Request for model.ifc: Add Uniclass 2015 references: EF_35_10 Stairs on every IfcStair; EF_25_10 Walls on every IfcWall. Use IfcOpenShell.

First a look at what the model holds.

```python
import ifcopenshell

model = ifcopenshell.open("model.ifc")
print(model.schema)
print("classifications:", [c.Name for c in model.by_type("IfcClassification")])
for ifc_class in ("IfcDoor", "IfcRoof", "IfcStair", "IfcWall", "IfcWindow"):
    print(ifc_class, len(model.by_type(ifc_class)))
```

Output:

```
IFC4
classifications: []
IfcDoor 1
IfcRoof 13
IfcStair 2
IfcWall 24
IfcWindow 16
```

```python
import ifcopenshell
import ifcopenshell.api.classification

model = ifcopenshell.open("model.ifc")

system = ifcopenshell.api.classification.add_classification(model, classification="Uniclass 2015")

codes = {
    "IfcStair": ("EF_35_10", "Stairs"),
    "IfcWall": ("EF_25_10", "Walls"),
}
for ifc_class, (code, name) in codes.items():
    products = model.by_type(ifc_class)
    ifcopenshell.api.classification.add_reference(
        model, products=products, classification=system, identification=code, name=name
    )
    print(code, len(products))

model.write("model_rev.ifc")
```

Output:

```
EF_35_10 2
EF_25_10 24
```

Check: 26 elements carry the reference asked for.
